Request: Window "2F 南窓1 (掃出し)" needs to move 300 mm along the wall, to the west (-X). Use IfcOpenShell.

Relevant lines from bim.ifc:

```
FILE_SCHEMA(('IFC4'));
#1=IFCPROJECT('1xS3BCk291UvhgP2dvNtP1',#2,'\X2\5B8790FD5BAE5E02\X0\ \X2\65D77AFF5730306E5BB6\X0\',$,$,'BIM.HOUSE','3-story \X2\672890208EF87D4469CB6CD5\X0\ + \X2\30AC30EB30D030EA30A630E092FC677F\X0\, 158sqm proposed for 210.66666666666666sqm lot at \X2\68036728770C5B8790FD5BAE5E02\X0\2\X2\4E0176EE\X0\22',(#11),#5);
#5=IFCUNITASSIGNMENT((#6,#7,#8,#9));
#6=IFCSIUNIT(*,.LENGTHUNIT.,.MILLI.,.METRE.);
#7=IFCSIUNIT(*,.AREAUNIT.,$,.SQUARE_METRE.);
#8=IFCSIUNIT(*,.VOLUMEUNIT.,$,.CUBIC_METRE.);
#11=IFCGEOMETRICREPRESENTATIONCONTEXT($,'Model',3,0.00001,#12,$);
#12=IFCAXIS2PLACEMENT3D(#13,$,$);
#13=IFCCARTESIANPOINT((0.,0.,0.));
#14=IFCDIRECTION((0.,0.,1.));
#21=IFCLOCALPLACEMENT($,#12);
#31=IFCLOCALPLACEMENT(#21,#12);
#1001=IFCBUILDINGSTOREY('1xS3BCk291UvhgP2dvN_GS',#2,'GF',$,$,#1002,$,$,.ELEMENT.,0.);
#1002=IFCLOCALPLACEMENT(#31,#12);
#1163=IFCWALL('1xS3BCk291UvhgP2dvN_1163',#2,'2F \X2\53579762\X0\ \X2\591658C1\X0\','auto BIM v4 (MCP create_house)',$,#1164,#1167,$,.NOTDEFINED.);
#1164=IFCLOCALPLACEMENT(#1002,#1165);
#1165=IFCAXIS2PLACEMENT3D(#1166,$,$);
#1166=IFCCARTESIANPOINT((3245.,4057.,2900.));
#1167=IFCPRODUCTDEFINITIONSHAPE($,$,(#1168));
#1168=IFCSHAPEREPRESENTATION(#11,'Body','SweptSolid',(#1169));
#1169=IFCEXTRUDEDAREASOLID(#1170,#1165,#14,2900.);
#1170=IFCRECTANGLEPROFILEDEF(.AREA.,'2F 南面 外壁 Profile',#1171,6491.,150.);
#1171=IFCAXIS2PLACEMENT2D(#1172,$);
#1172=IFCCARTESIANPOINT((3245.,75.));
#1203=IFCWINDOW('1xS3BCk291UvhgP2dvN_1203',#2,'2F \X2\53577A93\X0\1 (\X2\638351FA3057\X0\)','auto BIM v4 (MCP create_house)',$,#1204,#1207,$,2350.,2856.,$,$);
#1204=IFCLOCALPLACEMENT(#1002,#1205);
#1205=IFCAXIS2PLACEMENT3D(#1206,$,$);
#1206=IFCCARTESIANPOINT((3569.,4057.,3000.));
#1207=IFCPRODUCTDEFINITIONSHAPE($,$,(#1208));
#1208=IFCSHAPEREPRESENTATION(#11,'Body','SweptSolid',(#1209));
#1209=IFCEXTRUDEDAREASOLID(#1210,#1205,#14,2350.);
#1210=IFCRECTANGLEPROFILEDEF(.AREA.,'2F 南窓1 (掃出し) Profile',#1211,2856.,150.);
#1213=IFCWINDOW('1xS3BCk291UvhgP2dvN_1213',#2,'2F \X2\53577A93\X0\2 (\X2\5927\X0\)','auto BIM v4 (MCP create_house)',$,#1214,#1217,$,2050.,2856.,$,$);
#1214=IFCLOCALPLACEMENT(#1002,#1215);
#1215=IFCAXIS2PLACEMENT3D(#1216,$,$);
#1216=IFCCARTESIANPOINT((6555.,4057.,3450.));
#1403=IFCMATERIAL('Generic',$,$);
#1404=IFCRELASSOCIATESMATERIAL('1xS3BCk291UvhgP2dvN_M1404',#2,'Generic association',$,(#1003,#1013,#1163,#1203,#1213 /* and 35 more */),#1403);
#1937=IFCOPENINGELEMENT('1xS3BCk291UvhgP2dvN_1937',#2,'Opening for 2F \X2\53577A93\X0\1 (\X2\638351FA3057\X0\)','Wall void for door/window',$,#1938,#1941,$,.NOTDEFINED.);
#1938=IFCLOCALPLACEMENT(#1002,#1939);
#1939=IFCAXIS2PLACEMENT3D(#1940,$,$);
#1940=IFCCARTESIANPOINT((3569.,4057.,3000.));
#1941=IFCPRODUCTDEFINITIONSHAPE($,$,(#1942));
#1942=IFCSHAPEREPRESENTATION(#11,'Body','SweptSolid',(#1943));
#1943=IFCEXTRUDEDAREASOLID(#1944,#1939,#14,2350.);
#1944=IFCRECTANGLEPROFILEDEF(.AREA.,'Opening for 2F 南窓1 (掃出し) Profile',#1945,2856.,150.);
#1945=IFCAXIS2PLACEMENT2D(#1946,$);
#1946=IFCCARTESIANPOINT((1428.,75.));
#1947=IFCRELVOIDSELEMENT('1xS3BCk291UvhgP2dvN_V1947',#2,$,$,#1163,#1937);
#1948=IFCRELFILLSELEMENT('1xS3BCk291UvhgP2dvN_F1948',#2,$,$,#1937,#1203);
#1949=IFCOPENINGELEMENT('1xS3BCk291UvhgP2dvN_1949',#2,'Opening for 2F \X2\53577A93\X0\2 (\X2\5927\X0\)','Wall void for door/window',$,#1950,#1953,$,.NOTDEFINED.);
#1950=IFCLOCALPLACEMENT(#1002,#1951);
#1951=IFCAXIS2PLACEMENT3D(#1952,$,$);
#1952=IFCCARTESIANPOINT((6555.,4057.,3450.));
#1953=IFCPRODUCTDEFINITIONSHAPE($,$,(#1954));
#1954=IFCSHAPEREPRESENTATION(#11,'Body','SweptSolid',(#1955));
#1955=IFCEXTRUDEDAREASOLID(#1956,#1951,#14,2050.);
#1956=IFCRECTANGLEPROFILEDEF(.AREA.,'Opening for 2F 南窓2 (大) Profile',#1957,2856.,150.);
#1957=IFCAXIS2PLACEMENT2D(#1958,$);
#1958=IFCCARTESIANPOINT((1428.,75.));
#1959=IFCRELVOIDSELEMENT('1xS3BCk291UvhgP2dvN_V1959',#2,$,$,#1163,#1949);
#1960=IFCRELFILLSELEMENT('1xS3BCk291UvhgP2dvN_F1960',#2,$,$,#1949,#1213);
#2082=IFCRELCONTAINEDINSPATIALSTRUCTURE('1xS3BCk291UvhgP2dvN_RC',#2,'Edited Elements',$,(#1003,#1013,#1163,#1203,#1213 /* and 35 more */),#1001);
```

```python
import ifcopenshell
import ifcopenshell.api.geometry
import ifcopenshell.util.placement
import ifcopenshell.util.unit

model = ifcopenshell.open("bim.ifc")
unit_scale = ifcopenshell.util.unit.calculate_unit_scale(model)

window = model.by_guid("1xS3BCk291UvhgP2dvN_1203")
opening = window.FillsVoids[0].RelatingOpeningElement
wall = opening.VoidsElements[0].RelatingBuildingElement

wall_matrix = ifcopenshell.util.placement.get_local_placement(wall.ObjectPlacement)
shift = wall_matrix[:3, 0] * -0.3 / unit_scale
before = ifcopenshell.util.placement.get_local_placement(window.ObjectPlacement)[:3, 3].copy()

# The window is not placed relative to its opening, so move both.
for product in (opening, window):
    matrix = ifcopenshell.util.placement.get_local_placement(product.ObjectPlacement)
    matrix[:3, 3] += shift
    ifcopenshell.api.geometry.edit_object_placement(model, product=product, matrix=matrix, is_si=False)

after = ifcopenshell.util.placement.get_local_placement(window.ObjectPlacement)[:3, 3]
print("window moved by", (after - before).round(3) + 0.0)

model.write("bim-out.ifc")
```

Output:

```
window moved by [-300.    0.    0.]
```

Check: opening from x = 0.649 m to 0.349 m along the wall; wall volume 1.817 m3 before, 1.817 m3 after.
